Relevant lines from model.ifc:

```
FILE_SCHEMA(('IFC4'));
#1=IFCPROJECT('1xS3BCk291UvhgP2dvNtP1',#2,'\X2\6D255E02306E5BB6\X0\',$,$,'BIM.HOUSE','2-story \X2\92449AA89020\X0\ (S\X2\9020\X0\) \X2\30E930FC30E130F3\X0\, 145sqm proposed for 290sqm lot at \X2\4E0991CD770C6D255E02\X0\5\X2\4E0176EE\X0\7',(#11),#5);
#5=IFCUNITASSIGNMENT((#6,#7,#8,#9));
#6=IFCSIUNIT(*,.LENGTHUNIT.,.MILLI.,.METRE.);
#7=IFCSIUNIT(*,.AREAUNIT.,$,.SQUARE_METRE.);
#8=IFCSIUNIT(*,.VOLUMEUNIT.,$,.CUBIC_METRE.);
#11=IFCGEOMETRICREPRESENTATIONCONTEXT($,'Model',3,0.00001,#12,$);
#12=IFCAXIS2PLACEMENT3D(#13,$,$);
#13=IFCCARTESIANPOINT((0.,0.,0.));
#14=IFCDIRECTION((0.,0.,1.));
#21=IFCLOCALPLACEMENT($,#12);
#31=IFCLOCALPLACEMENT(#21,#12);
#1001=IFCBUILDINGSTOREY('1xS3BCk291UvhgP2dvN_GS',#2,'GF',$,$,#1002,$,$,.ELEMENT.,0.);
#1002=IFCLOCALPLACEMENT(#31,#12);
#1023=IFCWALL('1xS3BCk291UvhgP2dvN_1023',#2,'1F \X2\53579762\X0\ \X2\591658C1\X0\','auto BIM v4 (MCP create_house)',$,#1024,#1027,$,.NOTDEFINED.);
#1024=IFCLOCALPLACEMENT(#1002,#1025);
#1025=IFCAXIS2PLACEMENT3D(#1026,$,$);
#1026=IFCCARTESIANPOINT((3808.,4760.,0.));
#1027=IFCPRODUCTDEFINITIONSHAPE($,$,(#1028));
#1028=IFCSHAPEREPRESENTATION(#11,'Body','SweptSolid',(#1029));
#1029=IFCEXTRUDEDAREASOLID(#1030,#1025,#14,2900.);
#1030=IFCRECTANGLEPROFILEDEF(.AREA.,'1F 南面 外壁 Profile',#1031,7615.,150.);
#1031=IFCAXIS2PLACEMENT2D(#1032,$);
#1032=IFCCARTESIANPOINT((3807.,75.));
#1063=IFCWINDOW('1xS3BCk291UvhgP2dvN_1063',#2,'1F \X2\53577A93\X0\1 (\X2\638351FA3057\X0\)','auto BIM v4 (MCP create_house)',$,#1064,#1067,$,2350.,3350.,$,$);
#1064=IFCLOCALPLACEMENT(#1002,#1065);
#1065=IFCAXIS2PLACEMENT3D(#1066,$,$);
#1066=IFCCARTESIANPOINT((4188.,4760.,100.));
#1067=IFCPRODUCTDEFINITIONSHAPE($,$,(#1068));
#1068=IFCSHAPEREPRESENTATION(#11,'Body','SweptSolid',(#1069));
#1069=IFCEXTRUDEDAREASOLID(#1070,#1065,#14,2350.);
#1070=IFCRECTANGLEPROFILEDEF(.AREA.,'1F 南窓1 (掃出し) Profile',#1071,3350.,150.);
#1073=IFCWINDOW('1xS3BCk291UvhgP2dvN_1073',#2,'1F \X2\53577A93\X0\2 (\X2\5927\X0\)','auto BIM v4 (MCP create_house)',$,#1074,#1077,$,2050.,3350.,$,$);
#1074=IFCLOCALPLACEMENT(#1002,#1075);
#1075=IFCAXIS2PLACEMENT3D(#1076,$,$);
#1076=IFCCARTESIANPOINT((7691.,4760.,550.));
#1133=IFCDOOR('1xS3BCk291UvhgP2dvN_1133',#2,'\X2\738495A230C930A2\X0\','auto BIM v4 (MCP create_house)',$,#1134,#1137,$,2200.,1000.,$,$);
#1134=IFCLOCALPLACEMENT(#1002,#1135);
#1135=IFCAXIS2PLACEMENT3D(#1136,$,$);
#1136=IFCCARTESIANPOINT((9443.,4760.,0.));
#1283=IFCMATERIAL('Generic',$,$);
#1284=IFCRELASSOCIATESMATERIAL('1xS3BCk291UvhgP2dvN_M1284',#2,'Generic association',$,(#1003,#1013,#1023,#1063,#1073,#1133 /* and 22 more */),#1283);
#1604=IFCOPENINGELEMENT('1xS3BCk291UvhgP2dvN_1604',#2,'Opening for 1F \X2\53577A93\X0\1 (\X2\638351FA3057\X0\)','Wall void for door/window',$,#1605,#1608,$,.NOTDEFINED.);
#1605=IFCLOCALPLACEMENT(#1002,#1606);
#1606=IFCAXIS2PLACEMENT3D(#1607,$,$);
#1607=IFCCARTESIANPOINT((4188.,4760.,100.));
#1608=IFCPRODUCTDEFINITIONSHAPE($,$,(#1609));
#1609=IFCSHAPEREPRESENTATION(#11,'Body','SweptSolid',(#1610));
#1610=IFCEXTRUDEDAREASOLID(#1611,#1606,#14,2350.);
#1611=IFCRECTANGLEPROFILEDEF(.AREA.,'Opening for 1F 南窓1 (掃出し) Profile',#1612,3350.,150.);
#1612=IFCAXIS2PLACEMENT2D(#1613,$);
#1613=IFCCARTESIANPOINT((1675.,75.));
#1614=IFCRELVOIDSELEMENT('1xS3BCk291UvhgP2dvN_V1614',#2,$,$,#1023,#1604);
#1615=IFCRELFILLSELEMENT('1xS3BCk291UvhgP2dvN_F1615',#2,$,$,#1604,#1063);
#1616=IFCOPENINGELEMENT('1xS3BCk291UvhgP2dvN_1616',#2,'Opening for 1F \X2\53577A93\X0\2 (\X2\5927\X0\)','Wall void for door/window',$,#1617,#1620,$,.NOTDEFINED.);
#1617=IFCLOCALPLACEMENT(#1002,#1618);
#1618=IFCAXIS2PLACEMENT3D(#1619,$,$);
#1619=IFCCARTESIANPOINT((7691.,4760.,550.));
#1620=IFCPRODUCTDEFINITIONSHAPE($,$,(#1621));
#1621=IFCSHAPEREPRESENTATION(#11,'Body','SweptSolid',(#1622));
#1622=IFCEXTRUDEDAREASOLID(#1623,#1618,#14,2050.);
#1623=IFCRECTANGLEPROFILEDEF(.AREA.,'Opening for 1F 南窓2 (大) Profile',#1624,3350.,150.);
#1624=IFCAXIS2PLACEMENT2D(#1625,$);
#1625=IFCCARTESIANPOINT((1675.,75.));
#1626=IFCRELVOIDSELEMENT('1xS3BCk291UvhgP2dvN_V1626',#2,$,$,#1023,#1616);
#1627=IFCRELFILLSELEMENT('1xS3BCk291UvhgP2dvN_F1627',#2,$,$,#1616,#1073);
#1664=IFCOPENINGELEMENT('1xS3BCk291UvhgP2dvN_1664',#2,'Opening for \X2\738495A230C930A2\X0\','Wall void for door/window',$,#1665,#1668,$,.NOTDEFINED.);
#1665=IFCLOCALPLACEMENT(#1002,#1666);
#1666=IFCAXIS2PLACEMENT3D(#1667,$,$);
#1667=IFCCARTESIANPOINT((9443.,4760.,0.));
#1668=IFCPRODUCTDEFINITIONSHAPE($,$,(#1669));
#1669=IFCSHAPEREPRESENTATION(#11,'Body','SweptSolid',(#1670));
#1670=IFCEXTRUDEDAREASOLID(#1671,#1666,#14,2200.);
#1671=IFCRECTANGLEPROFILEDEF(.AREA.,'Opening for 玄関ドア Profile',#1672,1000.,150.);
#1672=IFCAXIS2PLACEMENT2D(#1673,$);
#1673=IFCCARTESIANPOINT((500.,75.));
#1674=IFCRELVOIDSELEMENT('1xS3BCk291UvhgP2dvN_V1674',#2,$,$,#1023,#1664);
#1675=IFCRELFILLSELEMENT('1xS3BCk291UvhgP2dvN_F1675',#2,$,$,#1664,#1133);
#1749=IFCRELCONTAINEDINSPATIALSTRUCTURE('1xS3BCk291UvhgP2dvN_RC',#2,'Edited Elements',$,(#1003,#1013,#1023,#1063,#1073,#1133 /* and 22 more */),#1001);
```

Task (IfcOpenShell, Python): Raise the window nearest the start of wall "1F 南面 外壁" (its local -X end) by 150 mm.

```python
import numpy as np
import ifcopenshell
import ifcopenshell.api.geometry
import ifcopenshell.util.placement
import ifcopenshell.util.unit

model = ifcopenshell.open("model.ifc")
unit_scale = ifcopenshell.util.unit.calculate_unit_scale(model)

window = model.by_guid("1xS3BCk291UvhgP2dvN_1063")
opening = window.FillsVoids[0].RelatingOpeningElement
dz = 0.15 / unit_scale

shift = np.array([0.0, 0.0, dz])
# The window is not placed relative to its opening, so move both.
for product in (opening, window):
    matrix = ifcopenshell.util.placement.get_local_placement(product.ObjectPlacement)
    matrix[:3, 3] += shift
    ifcopenshell.api.geometry.edit_object_placement(model, product=product, matrix=matrix, is_si=False)

print(f"moved by {dz * unit_scale:+.3f} m")

model.write("model_updated.ifc")
```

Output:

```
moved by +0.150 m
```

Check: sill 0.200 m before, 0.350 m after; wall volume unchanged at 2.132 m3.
